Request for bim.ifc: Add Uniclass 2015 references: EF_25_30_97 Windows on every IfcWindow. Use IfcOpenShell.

First a look at what the model holds.

```python
import ifcopenshell

model = ifcopenshell.open("bim.ifc")
print(model.schema)
print("classifications:", [c.Name for c in model.by_type("IfcClassification")])
for ifc_class in ("IfcDoor", "IfcRoof", "IfcStair", "IfcWall", "IfcWindow"):
    print(ifc_class, len(model.by_type(ifc_class)))
```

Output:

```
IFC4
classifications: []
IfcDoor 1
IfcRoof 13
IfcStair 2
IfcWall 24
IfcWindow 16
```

```python
import ifcopenshell
import ifcopenshell.api.classification

model = ifcopenshell.open("bim.ifc")

system = ifcopenshell.api.classification.add_classification(model, classification="Uniclass 2015")

codes = {
    "IfcWindow": ("EF_25_30_97", "Windows"),
}
for ifc_class, (code, name) in codes.items():
    products = model.by_type(ifc_class)
    ifcopenshell.api.classification.add_reference(
        model, products=products, classification=system, identification=code, name=name
    )
    print(code, len(products))

model.write("bim_edited.ifc")
```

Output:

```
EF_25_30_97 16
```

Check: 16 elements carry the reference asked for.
